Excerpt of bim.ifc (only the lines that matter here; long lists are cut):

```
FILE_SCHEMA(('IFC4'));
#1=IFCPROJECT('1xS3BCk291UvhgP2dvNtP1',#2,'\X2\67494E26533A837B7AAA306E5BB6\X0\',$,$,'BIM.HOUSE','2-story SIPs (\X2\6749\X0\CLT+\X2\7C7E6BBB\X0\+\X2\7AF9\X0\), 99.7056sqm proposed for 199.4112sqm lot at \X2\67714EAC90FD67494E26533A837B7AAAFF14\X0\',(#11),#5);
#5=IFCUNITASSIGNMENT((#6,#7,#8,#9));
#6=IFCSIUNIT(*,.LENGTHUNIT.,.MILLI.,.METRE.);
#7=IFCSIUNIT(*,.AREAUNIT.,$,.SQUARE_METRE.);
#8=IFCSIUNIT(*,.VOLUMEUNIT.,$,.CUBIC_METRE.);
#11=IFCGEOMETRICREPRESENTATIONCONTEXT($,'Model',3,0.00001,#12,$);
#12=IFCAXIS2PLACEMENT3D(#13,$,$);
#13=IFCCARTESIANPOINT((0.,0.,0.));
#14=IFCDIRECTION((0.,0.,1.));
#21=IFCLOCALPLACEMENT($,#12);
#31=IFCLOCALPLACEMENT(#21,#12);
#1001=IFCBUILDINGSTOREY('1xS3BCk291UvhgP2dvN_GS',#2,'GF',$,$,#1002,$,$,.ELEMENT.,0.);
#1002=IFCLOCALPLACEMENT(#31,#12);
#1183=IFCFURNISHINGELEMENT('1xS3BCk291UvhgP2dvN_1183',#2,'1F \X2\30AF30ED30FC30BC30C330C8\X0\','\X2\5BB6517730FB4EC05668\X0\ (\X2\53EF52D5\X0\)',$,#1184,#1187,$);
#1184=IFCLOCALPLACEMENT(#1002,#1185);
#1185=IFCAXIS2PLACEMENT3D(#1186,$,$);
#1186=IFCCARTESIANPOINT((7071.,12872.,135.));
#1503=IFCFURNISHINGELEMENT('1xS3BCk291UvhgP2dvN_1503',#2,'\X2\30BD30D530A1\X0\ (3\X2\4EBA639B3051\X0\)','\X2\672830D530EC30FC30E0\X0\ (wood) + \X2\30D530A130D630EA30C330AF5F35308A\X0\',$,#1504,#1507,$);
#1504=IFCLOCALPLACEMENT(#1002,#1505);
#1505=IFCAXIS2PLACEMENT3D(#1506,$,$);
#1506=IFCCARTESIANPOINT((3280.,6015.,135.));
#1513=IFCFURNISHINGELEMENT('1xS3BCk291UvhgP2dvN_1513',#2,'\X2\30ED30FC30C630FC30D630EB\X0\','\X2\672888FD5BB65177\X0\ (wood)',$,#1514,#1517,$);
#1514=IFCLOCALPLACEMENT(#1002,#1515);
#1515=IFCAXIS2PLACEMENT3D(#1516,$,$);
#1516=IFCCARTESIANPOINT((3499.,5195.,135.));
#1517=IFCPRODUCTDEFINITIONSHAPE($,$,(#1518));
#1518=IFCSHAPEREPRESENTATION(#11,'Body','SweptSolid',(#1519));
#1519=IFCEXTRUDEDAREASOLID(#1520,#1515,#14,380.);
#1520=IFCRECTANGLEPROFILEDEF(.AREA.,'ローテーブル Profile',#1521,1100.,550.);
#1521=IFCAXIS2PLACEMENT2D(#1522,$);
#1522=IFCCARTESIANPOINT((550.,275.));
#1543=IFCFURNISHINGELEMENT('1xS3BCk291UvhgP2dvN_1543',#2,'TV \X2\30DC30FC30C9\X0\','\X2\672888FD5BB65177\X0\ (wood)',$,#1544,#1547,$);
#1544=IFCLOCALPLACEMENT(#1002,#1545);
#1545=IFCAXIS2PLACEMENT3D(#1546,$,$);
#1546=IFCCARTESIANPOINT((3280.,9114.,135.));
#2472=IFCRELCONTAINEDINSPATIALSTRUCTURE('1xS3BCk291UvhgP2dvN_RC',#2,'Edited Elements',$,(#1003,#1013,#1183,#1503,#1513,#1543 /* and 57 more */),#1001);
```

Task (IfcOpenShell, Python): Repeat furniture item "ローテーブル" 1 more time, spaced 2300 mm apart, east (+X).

```python
import numpy as np
import ifcopenshell
import ifcopenshell.api.geometry
import ifcopenshell.api.root
import ifcopenshell.util.element
import ifcopenshell.util.placement

model = ifcopenshell.open("bim.ifc")


def reuse_history(source, copy):
    """copy_class also copies each property set's owner history, people and application; keep the originals."""
    for rel in copy.IsDefinedBy:
        if rel.is_a("IfcRelDefinesByProperties") and (history := rel.RelatingPropertyDefinition.OwnerHistory):
            rel.RelatingPropertyDefinition.OwnerHistory = source.OwnerHistory
            ifcopenshell.util.element.remove_deep2(model, history)


source = model.by_guid("1xS3BCk291UvhgP2dvN_1513")
base = ifcopenshell.util.placement.get_local_placement(source.ObjectPlacement)
step = np.array([1.0, 0.0, 0.0]) * 2300.0

for i in range(1, 2):
    copy = ifcopenshell.api.root.copy_class(model, product=source)
    copy.Representation = ifcopenshell.util.element.copy_deep(
        model, source.Representation, exclude=["IfcGeometricRepresentationContext", "IfcRepresentationMap"]
    )
    reuse_history(source, copy)
    matrix = base.copy()
    matrix[:3, 3] += i * step
    print("added at", matrix[:3, 3].round(3) + 0.0)
    ifcopenshell.api.geometry.edit_object_placement(model, product=copy, matrix=matrix, is_si=False)

model.write("bim_updated.ifc")
```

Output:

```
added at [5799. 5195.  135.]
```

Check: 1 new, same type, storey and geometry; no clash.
